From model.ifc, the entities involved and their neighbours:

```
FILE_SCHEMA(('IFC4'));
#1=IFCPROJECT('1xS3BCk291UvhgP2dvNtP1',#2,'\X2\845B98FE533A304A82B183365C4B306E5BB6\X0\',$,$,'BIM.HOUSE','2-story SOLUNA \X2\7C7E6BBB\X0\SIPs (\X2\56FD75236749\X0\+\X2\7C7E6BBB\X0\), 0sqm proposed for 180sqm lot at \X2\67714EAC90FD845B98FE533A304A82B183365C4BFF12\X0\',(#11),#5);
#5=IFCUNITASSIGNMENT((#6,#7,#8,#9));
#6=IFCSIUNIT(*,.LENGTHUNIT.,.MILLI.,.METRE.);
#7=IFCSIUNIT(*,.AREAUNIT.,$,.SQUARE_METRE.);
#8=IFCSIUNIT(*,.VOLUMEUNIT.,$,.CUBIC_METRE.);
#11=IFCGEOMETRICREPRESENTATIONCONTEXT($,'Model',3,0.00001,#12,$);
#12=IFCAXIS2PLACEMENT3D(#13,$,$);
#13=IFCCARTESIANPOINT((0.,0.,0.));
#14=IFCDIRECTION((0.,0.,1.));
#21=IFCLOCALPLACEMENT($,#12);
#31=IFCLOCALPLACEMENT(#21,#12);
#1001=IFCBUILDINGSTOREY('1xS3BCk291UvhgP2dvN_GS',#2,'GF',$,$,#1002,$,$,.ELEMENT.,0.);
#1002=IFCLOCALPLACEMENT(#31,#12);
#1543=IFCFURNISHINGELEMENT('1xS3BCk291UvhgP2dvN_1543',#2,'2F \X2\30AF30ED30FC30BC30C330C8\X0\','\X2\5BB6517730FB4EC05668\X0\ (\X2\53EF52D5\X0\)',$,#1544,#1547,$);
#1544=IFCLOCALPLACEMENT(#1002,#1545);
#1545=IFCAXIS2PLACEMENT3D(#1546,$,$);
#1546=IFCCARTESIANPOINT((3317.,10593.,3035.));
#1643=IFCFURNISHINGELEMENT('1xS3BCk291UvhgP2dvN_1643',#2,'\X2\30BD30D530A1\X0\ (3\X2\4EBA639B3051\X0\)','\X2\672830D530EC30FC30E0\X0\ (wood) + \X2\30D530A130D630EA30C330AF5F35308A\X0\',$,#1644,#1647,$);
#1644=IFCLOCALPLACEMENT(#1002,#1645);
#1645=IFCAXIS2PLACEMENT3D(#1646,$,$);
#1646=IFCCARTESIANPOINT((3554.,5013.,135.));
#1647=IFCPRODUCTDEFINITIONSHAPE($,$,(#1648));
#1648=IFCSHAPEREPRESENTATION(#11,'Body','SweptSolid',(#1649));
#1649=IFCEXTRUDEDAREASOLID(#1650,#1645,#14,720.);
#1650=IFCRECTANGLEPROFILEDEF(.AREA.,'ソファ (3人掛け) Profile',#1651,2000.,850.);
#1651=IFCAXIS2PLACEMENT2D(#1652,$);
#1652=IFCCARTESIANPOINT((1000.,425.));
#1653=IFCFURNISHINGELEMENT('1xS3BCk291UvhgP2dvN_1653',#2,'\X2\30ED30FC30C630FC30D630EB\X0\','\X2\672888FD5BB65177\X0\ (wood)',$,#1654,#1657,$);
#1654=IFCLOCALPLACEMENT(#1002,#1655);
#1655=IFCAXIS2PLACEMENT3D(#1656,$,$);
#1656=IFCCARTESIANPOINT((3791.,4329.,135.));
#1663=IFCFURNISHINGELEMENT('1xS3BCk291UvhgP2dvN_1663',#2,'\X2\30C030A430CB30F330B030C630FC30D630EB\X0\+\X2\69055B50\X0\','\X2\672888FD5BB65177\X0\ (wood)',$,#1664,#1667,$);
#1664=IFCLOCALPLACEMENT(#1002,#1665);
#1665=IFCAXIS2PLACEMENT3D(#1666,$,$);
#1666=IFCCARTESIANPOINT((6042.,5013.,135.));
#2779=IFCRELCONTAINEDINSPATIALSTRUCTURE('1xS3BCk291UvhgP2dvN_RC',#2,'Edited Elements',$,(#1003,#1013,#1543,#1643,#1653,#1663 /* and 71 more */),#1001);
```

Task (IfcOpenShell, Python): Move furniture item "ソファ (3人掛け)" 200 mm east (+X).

```python
import ifcopenshell
import ifcopenshell.api.geometry
import ifcopenshell.util.placement
import ifcopenshell.util.unit

model = ifcopenshell.open("model.ifc")
unit_scale = ifcopenshell.util.unit.calculate_unit_scale(model)

item = model.by_guid("1xS3BCk291UvhgP2dvN_1643")
matrix = ifcopenshell.util.placement.get_local_placement(item.ObjectPlacement)
matrix[0, 3] += 0.2 / unit_scale
ifcopenshell.api.geometry.edit_object_placement(model, product=item, matrix=matrix, is_si=False)

print(ifcopenshell.util.placement.get_local_placement(item.ObjectPlacement).round(3) + 0.0)

model.write("model-out.ifc")
```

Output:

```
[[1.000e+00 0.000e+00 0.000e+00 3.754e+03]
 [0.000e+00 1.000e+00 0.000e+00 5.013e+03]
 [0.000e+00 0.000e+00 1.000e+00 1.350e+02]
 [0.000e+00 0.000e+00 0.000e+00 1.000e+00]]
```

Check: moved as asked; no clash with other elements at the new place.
